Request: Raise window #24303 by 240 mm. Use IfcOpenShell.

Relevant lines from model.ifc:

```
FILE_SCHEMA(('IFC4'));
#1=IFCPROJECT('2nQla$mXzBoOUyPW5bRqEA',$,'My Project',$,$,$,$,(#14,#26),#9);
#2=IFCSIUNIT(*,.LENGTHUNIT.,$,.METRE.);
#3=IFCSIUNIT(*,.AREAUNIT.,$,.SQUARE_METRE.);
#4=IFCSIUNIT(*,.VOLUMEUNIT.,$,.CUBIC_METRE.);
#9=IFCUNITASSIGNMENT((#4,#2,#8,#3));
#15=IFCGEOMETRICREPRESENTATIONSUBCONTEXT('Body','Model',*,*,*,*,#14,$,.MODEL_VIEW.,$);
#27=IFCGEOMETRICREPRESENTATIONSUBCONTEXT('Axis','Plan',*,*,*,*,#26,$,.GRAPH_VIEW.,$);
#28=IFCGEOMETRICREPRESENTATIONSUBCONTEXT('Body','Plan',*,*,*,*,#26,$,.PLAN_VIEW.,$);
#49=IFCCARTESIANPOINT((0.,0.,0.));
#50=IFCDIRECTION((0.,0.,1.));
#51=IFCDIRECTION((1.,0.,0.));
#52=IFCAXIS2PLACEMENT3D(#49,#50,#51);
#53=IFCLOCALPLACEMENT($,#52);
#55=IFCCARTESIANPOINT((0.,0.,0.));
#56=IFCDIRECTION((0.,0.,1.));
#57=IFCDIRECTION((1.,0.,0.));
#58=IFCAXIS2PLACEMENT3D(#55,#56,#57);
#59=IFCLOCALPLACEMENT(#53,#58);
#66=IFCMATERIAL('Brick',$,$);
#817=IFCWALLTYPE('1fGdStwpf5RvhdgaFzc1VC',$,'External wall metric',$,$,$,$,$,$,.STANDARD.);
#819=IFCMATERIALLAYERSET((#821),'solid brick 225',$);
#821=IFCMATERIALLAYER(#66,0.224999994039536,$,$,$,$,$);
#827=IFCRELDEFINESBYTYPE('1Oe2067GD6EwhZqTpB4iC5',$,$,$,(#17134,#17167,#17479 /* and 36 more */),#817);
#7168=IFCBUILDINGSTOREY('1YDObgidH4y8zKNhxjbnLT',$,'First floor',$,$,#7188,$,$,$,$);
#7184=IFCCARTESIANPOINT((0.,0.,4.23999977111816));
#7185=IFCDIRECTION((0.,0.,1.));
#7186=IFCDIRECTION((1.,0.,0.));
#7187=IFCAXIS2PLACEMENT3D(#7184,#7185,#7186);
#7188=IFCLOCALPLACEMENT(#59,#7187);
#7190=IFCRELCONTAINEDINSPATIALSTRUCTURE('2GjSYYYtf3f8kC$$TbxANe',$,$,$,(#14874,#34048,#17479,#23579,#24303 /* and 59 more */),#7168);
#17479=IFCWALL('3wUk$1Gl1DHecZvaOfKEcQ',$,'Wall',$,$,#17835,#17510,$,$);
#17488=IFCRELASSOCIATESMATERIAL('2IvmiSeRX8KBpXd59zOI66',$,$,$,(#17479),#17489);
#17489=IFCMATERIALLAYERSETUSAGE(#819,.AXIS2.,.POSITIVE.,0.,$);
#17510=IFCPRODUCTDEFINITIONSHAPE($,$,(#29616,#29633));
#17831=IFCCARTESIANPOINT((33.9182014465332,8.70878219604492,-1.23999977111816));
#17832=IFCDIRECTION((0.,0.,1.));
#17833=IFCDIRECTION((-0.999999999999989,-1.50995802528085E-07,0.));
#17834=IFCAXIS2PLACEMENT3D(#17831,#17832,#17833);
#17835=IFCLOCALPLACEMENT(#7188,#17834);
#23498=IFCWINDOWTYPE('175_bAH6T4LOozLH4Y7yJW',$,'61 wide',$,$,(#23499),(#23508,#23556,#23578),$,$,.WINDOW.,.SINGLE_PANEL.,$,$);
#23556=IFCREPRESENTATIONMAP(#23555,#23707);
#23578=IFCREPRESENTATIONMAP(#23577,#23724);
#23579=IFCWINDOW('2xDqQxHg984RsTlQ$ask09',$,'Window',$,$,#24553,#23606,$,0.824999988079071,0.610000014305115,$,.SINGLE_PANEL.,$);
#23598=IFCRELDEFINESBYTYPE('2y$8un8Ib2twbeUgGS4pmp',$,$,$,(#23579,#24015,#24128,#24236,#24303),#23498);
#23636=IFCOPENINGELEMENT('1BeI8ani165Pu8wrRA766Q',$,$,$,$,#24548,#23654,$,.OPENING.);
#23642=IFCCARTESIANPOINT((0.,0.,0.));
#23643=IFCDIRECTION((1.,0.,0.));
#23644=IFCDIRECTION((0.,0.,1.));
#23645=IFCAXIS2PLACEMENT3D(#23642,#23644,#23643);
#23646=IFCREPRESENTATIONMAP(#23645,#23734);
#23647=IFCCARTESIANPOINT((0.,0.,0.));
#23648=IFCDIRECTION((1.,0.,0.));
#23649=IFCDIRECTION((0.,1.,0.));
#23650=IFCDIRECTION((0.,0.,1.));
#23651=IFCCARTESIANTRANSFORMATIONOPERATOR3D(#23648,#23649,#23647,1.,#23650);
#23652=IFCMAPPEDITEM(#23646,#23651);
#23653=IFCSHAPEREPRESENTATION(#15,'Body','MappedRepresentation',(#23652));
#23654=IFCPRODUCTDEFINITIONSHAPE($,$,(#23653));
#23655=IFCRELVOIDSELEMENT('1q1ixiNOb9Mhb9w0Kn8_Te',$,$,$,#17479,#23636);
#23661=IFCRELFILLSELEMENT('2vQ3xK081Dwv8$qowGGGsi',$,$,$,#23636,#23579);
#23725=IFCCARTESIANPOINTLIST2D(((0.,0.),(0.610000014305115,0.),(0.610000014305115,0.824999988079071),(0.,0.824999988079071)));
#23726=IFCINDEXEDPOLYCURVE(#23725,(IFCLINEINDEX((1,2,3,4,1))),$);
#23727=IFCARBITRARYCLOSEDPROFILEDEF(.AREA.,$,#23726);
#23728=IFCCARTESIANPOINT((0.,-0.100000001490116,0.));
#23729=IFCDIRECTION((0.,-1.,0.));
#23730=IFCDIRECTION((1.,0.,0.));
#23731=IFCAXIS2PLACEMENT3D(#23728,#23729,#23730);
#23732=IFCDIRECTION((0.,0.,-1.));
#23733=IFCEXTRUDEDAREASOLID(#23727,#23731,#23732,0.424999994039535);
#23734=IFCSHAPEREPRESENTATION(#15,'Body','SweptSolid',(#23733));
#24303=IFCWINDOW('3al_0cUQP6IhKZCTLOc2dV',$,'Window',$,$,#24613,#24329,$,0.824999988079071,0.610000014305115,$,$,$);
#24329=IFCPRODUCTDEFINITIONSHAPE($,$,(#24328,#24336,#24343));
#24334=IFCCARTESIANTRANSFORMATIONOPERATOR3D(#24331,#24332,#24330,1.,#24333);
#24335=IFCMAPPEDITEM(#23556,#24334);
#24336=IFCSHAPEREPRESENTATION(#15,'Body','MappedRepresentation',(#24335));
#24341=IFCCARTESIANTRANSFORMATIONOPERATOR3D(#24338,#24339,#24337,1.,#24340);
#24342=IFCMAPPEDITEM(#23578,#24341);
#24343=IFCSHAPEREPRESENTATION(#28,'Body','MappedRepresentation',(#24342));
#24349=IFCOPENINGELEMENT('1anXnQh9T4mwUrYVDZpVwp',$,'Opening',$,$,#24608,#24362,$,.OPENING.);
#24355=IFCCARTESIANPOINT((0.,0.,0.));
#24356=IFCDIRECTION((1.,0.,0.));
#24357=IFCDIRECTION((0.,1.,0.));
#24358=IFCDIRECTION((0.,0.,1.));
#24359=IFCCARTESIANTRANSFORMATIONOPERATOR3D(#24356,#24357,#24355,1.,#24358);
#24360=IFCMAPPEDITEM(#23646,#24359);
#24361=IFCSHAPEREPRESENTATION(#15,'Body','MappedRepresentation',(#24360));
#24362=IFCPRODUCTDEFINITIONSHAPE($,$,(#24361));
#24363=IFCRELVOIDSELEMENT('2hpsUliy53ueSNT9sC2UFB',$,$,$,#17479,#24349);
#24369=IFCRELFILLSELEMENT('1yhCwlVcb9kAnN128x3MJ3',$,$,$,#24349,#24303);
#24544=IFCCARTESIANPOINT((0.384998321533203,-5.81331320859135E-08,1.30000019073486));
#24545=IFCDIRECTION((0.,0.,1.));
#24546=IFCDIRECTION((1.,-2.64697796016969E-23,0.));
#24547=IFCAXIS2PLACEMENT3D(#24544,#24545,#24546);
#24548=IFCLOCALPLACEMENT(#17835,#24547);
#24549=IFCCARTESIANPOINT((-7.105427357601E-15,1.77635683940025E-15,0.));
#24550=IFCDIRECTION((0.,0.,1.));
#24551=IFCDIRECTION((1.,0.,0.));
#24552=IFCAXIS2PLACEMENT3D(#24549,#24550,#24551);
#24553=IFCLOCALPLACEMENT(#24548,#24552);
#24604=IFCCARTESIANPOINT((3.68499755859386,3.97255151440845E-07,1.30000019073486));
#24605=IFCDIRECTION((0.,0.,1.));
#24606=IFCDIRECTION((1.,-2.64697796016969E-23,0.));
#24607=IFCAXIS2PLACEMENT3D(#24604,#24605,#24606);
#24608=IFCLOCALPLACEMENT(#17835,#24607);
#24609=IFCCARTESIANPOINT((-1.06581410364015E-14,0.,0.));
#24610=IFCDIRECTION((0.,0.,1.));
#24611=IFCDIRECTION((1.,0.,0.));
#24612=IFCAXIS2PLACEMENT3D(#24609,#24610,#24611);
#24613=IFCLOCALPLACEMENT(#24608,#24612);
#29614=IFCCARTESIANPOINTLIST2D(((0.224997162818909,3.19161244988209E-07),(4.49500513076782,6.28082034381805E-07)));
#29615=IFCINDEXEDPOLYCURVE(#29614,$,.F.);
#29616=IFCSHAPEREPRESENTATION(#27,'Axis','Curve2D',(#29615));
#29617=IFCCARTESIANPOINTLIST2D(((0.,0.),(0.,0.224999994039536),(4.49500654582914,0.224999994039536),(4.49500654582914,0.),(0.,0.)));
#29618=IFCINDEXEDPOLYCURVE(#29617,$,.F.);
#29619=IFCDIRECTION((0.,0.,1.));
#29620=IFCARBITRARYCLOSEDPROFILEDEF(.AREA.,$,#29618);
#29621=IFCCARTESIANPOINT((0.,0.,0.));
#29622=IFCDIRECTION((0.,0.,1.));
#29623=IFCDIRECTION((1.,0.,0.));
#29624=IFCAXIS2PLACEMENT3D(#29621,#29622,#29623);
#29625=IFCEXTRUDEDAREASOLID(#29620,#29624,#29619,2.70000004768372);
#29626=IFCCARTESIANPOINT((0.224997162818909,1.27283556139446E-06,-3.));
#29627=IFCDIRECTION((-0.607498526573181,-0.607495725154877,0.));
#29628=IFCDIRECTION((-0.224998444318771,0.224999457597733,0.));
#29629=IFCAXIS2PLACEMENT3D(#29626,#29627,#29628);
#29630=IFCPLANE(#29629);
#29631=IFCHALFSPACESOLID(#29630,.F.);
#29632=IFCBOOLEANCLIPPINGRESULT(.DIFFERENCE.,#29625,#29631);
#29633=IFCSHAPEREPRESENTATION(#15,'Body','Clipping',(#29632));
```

```python
import numpy as np
import ifcopenshell
import ifcopenshell.api.geometry
import ifcopenshell.util.placement
import ifcopenshell.util.unit

model = ifcopenshell.open("model.ifc")
unit_scale = ifcopenshell.util.unit.calculate_unit_scale(model)

window = model.by_id(24303)
opening = window.FillsVoids[0].RelatingOpeningElement
dz = 0.24

shift = np.array([0.0, 0.0, dz])
# The window is placed relative to its opening, so it follows when the opening moves.
matrix = ifcopenshell.util.placement.get_local_placement(opening.ObjectPlacement)
matrix[:3, 3] += shift
ifcopenshell.api.geometry.edit_object_placement(
    model, product=opening, matrix=matrix, is_si=False, should_transform_children=True
)

print(f"moved by {dz * unit_scale:+.3f} m")

model.write("model_v2.ifc")
```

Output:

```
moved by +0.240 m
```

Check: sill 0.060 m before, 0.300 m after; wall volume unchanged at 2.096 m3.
